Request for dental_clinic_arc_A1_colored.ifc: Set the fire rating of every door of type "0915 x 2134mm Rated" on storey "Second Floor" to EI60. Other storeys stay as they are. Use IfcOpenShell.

First a look at what the model holds.

```python
import ifcopenshell
import ifcopenshell.util.element

model = ifcopenshell.open("dental_clinic_arc_A1_colored.ifc")
print(model.schema)
storey = next(s for s in model.by_type("IfcBuildingStorey") if s.Name == "Second Floor")
doors = [e for e in ifcopenshell.util.element.get_decomposition(storey) if e.is_a("IfcDoor")]
seen = {}
for e in doors:
    element_type = ifcopenshell.util.element.get_type(e)
    key = (element_type.Name if element_type != e and element_type else None, ifcopenshell.util.element.get_pset(e, "Pset_DoorCommon", "FireRating"))
    seen[key] = seen.get(key, 0) + 1
for (name, value), count in sorted(seen.items(), key=str):
    print(count, "x", name, "|", value)
```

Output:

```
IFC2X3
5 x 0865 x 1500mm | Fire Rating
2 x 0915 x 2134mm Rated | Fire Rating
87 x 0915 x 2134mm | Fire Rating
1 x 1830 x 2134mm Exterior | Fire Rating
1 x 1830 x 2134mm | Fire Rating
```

```python
import ifcopenshell
import ifcopenshell.api.pset
import ifcopenshell.util.element

model = ifcopenshell.open("dental_clinic_arc_A1_colored.ifc")

storey = next(s for s in model.by_type("IfcBuildingStorey") if s.Name == "Second Floor")
doors = [e for e in ifcopenshell.util.element.get_decomposition(storey) if e.is_a("IfcDoor")]

count = 0
for e in doors:
    element_type = ifcopenshell.util.element.get_type(e)
    if element_type in (None, e) or element_type.Name != "0915 x 2134mm Rated":
        continue
    # add_pset returns the element's existing set when there is one.
    pset = ifcopenshell.api.pset.add_pset(model, product=e, name="Pset_DoorCommon")
    ifcopenshell.api.pset.edit_pset(model, pset=pset, properties={"FireRating": "EI60"})
    count += 1

print(count, "doors updated")

model.write("dental_clinic_arc_A1_colored-out.ifc")
```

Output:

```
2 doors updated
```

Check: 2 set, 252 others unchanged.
